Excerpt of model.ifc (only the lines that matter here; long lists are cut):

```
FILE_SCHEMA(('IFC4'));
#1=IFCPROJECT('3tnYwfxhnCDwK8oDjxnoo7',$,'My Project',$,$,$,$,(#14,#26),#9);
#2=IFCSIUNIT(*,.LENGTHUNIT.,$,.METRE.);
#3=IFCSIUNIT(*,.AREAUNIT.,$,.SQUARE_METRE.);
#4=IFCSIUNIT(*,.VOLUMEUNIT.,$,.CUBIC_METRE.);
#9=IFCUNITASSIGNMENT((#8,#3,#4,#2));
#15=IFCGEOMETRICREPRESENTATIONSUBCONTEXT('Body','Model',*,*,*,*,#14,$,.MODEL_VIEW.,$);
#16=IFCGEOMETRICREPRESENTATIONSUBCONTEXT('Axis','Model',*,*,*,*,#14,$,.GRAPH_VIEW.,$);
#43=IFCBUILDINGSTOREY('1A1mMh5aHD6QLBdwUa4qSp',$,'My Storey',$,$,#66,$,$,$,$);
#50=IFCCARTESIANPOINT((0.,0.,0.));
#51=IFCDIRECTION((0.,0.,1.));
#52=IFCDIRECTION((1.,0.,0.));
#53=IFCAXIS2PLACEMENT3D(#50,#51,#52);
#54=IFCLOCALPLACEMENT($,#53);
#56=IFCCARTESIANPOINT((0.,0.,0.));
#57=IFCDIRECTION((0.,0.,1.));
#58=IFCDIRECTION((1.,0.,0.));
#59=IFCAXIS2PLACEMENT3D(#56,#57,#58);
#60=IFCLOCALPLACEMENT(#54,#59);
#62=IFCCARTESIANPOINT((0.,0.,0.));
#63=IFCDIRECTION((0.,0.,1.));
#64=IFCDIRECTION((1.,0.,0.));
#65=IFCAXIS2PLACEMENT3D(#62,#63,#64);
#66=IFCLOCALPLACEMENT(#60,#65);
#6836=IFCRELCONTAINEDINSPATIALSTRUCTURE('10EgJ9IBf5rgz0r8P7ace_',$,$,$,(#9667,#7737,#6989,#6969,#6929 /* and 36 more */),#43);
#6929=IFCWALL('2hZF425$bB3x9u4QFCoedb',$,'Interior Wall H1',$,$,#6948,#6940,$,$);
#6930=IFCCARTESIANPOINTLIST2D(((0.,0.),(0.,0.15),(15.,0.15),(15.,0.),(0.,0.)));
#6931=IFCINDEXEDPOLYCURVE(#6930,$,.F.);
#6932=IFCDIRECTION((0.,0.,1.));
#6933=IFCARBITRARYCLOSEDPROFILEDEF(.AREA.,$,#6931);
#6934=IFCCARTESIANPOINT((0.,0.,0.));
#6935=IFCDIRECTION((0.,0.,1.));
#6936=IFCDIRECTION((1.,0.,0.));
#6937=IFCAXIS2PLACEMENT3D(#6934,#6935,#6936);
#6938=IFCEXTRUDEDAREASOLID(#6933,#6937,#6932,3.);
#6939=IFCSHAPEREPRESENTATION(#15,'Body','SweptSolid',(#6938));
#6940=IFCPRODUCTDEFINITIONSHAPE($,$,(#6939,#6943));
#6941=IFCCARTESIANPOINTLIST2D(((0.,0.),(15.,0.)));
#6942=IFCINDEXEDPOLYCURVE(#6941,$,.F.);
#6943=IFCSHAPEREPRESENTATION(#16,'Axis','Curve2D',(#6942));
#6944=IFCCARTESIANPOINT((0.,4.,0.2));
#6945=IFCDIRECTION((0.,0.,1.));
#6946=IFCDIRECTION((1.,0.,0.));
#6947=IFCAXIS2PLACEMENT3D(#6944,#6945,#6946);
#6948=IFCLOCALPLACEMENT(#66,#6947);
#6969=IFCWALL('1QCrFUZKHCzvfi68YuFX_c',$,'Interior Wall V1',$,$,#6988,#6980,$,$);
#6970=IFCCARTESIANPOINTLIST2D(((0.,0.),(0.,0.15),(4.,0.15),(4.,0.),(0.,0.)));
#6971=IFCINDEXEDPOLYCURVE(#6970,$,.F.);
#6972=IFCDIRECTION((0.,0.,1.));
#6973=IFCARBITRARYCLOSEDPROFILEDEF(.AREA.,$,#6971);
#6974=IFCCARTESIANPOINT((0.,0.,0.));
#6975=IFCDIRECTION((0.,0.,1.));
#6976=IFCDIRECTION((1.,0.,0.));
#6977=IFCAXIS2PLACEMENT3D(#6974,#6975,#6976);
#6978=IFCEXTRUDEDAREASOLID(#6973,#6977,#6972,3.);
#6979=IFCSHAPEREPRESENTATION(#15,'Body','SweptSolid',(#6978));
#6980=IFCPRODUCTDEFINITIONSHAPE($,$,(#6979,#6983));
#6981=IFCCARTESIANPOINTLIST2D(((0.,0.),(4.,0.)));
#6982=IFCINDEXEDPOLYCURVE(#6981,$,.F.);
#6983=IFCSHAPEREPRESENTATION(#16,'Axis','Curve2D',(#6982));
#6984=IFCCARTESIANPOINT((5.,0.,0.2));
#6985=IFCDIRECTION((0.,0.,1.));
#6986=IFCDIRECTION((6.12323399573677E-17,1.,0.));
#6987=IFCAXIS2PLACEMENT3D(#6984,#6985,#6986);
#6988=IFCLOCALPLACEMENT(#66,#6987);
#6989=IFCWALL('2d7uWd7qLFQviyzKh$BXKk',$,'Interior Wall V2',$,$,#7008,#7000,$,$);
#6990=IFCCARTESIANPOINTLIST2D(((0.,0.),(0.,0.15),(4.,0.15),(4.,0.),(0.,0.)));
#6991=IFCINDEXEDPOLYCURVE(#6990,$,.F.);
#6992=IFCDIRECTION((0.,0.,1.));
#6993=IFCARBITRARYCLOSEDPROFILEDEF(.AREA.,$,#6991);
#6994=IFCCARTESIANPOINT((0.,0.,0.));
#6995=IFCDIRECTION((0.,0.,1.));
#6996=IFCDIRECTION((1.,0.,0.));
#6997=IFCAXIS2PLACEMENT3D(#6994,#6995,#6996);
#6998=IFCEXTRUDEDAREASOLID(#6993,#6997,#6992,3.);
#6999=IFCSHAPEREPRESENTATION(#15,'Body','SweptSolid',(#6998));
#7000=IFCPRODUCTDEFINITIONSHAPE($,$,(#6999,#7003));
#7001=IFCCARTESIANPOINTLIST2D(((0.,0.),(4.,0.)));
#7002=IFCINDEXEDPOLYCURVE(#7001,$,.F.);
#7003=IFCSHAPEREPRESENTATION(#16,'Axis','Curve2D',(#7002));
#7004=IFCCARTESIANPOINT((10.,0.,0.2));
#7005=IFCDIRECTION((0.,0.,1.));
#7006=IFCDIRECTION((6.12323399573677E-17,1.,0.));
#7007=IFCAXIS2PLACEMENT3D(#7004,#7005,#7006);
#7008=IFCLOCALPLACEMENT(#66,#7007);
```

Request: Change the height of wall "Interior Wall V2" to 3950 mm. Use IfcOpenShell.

```python
import ifcopenshell
import ifcopenshell.geom
import ifcopenshell.util.representation
import ifcopenshell.util.shape
import ifcopenshell.util.unit

model = ifcopenshell.open("model.ifc")
unit_scale = ifcopenshell.util.unit.calculate_unit_scale(model)
settings = ifcopenshell.geom.settings()


def volume(element):
    """Net volume in cubic metres, openings subtracted."""
    shape = ifcopenshell.geom.create_shape(settings, element)
    return ifcopenshell.util.shape.get_volume(shape.geometry)


wall = model.by_guid("2d7uWd7qLFQviyzKh$BXKk")
before = volume(wall)

body = ifcopenshell.util.representation.get_representation(wall, "Model", "Body")
solid = body.Items[0]
old_height = solid.Depth
solid.Depth = 3.95 / unit_scale
after = volume(wall)

print(f"height {old_height:g} -> {solid.Depth:g}, volume {before:.3f} -> {after:.3f} m3")

model.write("model_v2.ifc")
```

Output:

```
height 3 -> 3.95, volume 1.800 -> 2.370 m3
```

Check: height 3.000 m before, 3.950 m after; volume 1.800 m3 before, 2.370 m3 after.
